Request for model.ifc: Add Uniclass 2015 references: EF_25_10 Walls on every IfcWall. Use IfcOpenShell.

First a look at what the model holds.

```python
import ifcopenshell

model = ifcopenshell.open("model.ifc")
print(model.schema)
print("classifications:", [c.Name for c in model.by_type("IfcClassification")])
for ifc_class in ("IfcDoor", "IfcRoof", "IfcStair", "IfcWall", "IfcWindow"):
    print(ifc_class, len(model.by_type(ifc_class)))
```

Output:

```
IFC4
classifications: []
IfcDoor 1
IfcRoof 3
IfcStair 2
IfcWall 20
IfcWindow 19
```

```python
import ifcopenshell
import ifcopenshell.api.classification

model = ifcopenshell.open("model.ifc")

system = ifcopenshell.api.classification.add_classification(model, classification="Uniclass 2015")

codes = {
    "IfcWall": ("EF_25_10", "Walls"),
}
for ifc_class, (code, name) in codes.items():
    products = model.by_type(ifc_class)
    ifcopenshell.api.classification.add_reference(
        model, products=products, classification=system, identification=code, name=name
    )
    print(code, len(products))

model.write("model_updated.ifc")
```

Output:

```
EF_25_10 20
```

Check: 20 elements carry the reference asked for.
